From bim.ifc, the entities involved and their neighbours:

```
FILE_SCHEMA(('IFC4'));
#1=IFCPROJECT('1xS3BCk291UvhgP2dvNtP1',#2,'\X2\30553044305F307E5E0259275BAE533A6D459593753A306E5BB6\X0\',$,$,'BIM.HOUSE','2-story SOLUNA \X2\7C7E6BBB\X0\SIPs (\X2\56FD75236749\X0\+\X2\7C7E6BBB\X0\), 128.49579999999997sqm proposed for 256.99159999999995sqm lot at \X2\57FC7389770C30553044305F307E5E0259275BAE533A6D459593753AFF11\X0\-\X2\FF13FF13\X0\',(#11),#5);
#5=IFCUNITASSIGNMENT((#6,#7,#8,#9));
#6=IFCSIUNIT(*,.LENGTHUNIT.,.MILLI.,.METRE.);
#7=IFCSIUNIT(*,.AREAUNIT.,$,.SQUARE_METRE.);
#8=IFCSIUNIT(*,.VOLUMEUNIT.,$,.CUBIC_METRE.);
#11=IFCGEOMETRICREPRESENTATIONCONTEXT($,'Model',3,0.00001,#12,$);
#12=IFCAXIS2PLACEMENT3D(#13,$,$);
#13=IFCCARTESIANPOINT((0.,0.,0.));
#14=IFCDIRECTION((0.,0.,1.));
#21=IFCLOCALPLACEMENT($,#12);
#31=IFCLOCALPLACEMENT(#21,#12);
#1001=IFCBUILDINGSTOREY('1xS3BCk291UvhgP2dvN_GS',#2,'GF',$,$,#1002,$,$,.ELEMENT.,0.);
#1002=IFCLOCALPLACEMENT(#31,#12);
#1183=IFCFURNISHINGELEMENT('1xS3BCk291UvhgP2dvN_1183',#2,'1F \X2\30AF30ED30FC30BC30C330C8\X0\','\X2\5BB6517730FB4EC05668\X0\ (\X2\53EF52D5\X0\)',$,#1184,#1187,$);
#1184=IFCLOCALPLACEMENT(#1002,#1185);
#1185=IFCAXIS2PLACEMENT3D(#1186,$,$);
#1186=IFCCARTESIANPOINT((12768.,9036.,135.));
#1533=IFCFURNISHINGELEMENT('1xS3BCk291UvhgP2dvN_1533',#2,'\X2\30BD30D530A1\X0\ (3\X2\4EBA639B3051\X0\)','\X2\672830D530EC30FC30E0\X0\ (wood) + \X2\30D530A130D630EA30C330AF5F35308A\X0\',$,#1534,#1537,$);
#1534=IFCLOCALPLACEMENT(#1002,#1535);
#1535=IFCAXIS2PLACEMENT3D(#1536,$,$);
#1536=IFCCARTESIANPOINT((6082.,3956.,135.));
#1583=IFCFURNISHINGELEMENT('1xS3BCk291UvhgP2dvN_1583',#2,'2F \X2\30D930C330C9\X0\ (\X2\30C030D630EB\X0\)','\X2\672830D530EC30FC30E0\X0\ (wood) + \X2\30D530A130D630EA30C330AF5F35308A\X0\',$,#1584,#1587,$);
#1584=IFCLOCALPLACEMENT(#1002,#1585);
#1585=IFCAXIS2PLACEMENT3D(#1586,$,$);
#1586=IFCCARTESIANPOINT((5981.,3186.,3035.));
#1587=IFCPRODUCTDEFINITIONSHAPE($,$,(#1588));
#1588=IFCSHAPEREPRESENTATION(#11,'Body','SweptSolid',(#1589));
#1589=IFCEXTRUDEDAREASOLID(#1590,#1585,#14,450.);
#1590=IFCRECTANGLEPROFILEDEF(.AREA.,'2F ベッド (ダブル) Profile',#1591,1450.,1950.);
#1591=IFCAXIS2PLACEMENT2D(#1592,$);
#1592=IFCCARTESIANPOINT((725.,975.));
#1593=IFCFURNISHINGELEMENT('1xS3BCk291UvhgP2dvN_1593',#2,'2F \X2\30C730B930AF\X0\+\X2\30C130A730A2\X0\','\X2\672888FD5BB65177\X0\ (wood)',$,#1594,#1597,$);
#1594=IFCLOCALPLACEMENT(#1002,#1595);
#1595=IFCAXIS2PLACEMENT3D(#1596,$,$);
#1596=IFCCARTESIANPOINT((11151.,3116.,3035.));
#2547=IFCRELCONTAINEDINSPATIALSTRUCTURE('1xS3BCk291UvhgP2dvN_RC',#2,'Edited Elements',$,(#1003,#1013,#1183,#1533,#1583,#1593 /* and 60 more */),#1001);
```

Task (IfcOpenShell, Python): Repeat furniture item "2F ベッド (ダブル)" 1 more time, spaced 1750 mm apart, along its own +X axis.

```python
import ifcopenshell
import ifcopenshell.api.geometry
import ifcopenshell.api.root
import ifcopenshell.util.element
import ifcopenshell.util.placement
import ifcopenshell.util.unit

model = ifcopenshell.open("bim.ifc")
unit_scale = ifcopenshell.util.unit.calculate_unit_scale(model)


def reuse_history(source, copy):
    """copy_class also copies each property set's owner history, people and application; keep the originals."""
    for rel in copy.IsDefinedBy:
        if rel.is_a("IfcRelDefinesByProperties") and (history := rel.RelatingPropertyDefinition.OwnerHistory):
            rel.RelatingPropertyDefinition.OwnerHistory = source.OwnerHistory
            ifcopenshell.util.element.remove_deep2(model, history)


source = model.by_guid("1xS3BCk291UvhgP2dvN_1583")
base = ifcopenshell.util.placement.get_local_placement(source.ObjectPlacement)
step = base[:3, 0] * 1.75 / unit_scale

for i in range(1, 2):
    copy = ifcopenshell.api.root.copy_class(model, product=source)
    copy.Representation = ifcopenshell.util.element.copy_deep(
        model, source.Representation, exclude=["IfcGeometricRepresentationContext", "IfcRepresentationMap"]
    )
    reuse_history(source, copy)
    matrix = base.copy()
    matrix[:3, 3] += i * step
    print("added at", matrix[:3, 3].round(3) + 0.0)
    ifcopenshell.api.geometry.edit_object_placement(model, product=copy, matrix=matrix, is_si=False)

model.write("bim-out.ifc")
```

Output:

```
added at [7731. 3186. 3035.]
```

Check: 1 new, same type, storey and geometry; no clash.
